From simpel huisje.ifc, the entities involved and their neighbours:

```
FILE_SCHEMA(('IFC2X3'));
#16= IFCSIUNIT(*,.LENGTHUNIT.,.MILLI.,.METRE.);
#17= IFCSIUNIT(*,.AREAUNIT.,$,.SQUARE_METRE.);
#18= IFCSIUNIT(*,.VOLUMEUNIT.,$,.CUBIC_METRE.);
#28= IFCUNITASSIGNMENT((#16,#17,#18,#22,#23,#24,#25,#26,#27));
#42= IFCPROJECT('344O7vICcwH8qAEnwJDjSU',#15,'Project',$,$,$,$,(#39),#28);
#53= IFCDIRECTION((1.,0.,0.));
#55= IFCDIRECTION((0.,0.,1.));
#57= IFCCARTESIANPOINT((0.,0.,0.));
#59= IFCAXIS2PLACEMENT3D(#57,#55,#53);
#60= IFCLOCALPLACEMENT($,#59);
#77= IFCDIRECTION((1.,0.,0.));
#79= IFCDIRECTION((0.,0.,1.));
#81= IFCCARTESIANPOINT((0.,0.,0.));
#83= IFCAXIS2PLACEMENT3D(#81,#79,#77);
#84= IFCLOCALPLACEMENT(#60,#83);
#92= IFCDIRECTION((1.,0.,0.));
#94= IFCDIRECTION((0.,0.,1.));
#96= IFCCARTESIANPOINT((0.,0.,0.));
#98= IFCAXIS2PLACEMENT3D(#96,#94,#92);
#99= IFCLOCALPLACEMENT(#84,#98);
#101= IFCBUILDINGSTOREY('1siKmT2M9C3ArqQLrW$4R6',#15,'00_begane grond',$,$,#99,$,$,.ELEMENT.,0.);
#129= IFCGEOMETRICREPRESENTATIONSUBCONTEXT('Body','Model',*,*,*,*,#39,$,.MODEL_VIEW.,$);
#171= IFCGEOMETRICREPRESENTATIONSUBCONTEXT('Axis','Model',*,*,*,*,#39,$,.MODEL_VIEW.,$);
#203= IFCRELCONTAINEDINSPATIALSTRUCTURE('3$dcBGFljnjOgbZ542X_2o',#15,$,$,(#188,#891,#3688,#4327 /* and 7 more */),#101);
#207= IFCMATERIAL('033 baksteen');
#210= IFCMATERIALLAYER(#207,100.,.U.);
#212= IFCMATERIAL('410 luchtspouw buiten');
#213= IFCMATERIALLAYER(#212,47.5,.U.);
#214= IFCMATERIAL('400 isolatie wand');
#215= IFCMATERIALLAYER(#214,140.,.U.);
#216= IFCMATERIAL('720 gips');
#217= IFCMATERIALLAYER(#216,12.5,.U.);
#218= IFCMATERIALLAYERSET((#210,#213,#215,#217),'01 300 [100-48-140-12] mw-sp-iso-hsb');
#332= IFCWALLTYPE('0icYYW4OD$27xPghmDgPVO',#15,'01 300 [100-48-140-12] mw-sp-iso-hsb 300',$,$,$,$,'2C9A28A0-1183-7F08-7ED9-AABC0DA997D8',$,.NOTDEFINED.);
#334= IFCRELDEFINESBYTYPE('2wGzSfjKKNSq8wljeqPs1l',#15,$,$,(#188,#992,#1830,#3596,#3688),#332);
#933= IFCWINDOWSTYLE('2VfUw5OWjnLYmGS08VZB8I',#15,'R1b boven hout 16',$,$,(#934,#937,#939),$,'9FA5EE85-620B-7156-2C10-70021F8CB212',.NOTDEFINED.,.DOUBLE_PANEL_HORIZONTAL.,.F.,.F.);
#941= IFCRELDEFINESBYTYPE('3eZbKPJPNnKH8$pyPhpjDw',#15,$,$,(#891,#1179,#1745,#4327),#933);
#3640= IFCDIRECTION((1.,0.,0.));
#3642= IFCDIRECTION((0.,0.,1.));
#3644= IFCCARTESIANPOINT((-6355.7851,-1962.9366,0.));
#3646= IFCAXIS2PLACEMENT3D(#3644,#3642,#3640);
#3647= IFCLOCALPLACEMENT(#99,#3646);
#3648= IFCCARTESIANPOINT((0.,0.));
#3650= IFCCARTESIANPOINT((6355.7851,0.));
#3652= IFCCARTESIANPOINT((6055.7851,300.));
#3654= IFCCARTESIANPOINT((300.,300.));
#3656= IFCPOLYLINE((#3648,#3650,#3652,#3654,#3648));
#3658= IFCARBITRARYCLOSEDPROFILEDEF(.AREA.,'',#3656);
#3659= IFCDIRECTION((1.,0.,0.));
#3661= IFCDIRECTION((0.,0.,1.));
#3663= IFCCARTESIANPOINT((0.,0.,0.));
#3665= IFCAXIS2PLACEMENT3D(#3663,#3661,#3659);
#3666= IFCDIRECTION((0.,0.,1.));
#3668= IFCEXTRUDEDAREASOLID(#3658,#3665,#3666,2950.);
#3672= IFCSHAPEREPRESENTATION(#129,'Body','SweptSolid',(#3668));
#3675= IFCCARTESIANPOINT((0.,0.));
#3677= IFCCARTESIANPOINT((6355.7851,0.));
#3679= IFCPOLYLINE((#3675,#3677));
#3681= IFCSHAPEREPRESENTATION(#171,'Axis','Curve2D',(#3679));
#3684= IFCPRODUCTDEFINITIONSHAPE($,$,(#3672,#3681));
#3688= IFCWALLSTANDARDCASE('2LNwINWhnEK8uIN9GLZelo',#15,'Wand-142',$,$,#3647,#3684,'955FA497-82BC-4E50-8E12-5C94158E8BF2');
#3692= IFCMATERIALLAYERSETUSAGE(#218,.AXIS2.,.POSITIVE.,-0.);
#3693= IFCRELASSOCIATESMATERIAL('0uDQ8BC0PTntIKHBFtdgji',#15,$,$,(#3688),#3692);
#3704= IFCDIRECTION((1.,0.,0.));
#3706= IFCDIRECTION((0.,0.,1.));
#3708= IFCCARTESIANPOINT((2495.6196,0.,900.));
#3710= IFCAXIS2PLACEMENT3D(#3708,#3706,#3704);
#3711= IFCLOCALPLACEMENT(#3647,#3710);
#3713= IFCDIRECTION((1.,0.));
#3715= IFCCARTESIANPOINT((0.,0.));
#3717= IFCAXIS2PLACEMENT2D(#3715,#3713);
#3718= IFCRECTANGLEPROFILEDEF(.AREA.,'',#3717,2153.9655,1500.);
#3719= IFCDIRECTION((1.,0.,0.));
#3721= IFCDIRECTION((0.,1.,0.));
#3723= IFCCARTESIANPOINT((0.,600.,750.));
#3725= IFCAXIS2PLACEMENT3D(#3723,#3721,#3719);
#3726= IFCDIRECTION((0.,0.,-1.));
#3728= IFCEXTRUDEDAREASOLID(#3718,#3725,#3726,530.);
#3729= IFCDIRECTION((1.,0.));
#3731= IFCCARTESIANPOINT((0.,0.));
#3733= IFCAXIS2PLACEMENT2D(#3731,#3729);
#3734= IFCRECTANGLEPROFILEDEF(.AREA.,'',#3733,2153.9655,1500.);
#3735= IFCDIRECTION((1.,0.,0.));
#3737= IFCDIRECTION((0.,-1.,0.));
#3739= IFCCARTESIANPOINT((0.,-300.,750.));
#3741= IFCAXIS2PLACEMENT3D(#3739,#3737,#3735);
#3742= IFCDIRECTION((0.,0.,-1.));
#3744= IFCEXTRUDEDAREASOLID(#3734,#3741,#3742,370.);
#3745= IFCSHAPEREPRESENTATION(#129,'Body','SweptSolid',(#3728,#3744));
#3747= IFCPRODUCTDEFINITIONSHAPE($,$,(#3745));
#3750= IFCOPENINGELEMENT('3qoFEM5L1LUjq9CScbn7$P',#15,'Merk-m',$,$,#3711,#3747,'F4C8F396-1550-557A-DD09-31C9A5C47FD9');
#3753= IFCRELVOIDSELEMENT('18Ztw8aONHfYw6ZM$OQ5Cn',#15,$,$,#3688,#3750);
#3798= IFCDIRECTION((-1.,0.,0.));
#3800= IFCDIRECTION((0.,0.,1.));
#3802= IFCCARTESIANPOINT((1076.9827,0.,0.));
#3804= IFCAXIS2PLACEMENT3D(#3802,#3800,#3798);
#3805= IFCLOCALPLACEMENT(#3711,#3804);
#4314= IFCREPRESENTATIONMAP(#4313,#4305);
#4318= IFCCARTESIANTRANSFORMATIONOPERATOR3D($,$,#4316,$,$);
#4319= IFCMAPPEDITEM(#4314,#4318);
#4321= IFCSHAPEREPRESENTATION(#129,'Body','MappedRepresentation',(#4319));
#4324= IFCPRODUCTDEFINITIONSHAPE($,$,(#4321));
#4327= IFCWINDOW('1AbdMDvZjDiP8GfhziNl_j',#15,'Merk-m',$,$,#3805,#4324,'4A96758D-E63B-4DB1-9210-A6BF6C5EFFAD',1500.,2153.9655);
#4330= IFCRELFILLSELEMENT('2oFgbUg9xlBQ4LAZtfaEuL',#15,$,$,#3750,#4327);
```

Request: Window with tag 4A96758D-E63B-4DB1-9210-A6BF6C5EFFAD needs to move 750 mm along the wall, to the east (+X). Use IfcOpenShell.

```python
import ifcopenshell
import ifcopenshell.api.geometry
import ifcopenshell.util.placement
import ifcopenshell.util.unit

model = ifcopenshell.open("simpel huisje.ifc")
unit_scale = ifcopenshell.util.unit.calculate_unit_scale(model)

window = model.by_guid("1AbdMDvZjDiP8GfhziNl_j")
opening = window.FillsVoids[0].RelatingOpeningElement
wall = opening.VoidsElements[0].RelatingBuildingElement

wall_matrix = ifcopenshell.util.placement.get_local_placement(wall.ObjectPlacement)
shift = wall_matrix[:3, 0] * 0.75 / unit_scale
before = ifcopenshell.util.placement.get_local_placement(window.ObjectPlacement)[:3, 3].copy()

# The window is placed relative to its opening, so it follows when the opening moves.
matrix = ifcopenshell.util.placement.get_local_placement(opening.ObjectPlacement)
matrix[:3, 3] += shift
ifcopenshell.api.geometry.edit_object_placement(
    model, product=opening, matrix=matrix, is_si=False, should_transform_children=True
)

after = ifcopenshell.util.placement.get_local_placement(window.ObjectPlacement)[:3, 3]
print("window moved by", (after - before).round(3) + 0.0)

model.write("simpel huisje_edited.ifc")
```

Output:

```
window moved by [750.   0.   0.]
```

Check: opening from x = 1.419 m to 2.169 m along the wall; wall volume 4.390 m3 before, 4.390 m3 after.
